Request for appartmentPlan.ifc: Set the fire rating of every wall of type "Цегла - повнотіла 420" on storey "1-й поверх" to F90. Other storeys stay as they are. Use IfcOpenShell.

First a look at what the model holds.

```python
import ifcopenshell
import ifcopenshell.util.element

model = ifcopenshell.open("appartmentPlan.ifc")
print(model.schema)
storey = next(s for s in model.by_type("IfcBuildingStorey") if s.Name == "1-й поверх")
walls = [e for e in ifcopenshell.util.element.get_decomposition(storey) if e.is_a("IfcWall")]
seen = {}
for e in walls:
    element_type = ifcopenshell.util.element.get_type(e)
    key = (element_type.Name if element_type != e and element_type else None, ifcopenshell.util.element.get_pset(e, "Pset_WallCommon", "FireRating"))
    seen[key] = seen.get(key, 0) + 1
for (name, value), count in sorted(seen.items(), key=str):
    print(count, "x", name, "|", value)
```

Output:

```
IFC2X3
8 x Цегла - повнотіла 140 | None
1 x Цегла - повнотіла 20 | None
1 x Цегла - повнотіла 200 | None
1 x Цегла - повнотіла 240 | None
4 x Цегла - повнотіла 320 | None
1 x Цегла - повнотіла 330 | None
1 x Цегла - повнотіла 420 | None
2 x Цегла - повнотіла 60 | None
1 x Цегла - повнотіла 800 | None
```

```python
import ifcopenshell
import ifcopenshell.api.pset
import ifcopenshell.util.element

model = ifcopenshell.open("appartmentPlan.ifc")

storey = next(s for s in model.by_type("IfcBuildingStorey") if s.Name == "1-й поверх")
walls = [e for e in ifcopenshell.util.element.get_decomposition(storey) if e.is_a("IfcWall")]

count = 0
for e in walls:
    element_type = ifcopenshell.util.element.get_type(e)
    if element_type in (None, e) or element_type.Name != "Цегла - повнотіла 420":
        continue
    # add_pset returns the element's existing set when there is one.
    pset = ifcopenshell.api.pset.add_pset(model, product=e, name="Pset_WallCommon")
    ifcopenshell.api.pset.edit_pset(model, pset=pset, properties={"FireRating": "F90"})
    count += 1

print(count, "walls updated")

model.write("appartmentPlan-out.ifc")
```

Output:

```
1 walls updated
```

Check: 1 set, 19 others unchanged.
